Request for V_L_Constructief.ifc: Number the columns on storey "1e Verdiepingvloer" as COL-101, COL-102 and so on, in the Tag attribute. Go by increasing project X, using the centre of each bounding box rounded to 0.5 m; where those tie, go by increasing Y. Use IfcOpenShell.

First a look at what the model holds.

```python
import ifcopenshell
import ifcopenshell.util.element
import ifcopenshell.util.placement

model = ifcopenshell.open("V_L_Constructief.ifc")
print(model.schema)
storey = next(s for s in model.by_type("IfcBuildingStorey") if s.Name == "1e Verdiepingvloer")
columns = [e for e in ifcopenshell.util.element.get_decomposition(storey) if e.is_a("IfcColumn")]
for e in sorted(columns, key=lambda e: e.id()):
    origin = ifcopenshell.util.placement.get_local_placement(e.ObjectPlacement)[:3, 3]
    print(e.id(), e.Tag, e.Name, origin.round(2) + 0.0, sep=" | ")
```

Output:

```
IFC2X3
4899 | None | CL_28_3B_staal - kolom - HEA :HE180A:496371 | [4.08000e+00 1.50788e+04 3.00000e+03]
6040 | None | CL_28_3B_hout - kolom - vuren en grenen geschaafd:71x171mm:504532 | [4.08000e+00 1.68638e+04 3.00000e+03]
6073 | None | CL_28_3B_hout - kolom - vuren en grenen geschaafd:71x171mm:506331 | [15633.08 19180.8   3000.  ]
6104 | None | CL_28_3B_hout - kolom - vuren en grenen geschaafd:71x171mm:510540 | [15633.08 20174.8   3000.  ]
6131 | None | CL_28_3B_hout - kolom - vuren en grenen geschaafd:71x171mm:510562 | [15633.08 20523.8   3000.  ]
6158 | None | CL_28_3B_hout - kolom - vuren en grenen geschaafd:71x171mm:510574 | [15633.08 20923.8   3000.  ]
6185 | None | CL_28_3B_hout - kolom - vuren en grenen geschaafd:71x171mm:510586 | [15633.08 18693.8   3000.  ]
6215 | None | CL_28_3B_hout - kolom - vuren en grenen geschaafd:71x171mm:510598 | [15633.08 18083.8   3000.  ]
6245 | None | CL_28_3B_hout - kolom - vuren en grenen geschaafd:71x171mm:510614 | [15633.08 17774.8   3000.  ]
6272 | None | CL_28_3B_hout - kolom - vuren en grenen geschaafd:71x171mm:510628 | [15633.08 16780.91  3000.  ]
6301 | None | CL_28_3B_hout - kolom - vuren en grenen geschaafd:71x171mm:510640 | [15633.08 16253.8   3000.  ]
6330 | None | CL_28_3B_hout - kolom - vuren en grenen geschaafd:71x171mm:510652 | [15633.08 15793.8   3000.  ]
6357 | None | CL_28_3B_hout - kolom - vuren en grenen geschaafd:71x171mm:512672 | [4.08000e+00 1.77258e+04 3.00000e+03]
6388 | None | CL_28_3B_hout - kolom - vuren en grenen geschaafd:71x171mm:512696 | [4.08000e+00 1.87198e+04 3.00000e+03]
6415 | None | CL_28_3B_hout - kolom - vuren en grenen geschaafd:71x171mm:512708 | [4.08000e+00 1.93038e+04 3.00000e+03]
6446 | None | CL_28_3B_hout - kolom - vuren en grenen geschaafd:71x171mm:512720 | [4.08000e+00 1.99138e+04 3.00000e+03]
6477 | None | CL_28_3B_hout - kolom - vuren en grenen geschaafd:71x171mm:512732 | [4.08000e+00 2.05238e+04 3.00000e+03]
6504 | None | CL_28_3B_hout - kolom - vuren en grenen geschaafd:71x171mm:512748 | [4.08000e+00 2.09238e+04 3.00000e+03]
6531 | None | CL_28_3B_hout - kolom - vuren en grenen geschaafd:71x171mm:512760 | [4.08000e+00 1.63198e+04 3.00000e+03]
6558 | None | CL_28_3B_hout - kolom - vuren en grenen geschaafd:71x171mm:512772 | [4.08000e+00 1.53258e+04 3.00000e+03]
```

```python
import ifcopenshell
import ifcopenshell.geom
import ifcopenshell.util.element
import ifcopenshell.util.shape

model = ifcopenshell.open("V_L_Constructief.ifc")
settings = ifcopenshell.geom.settings()
settings.set("use-world-coords", True)


def centre(element):
    shape = ifcopenshell.geom.create_shape(settings, element)
    return ifcopenshell.util.shape.get_bbox_centroid(shape.geometry)


storey = next(s for s in model.by_type("IfcBuildingStorey") if s.Name == "1e Verdiepingvloer")
columns = [e for e in ifcopenshell.util.element.get_decomposition(storey) if e.is_a("IfcColumn")]

# Insertion points can sit at a corner or the storey origin, so sort by the geometry (in metres).
centres = {e: centre(e) for e in columns}
columns.sort(key=lambda e: (round(centres[e][0] / 0.5), centres[e][1]))

for i, e in enumerate(columns, start=1):
    number = f"COL-1{i:02d}"
    e.Tag = number
    print(e.id(), number)

model.write("V_L_Constructief_edited.ifc")
```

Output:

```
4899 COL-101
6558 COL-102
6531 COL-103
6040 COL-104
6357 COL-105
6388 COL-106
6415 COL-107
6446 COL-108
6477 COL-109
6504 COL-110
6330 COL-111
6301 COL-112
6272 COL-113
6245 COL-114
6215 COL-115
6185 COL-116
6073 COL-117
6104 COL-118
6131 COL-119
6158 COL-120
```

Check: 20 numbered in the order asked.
